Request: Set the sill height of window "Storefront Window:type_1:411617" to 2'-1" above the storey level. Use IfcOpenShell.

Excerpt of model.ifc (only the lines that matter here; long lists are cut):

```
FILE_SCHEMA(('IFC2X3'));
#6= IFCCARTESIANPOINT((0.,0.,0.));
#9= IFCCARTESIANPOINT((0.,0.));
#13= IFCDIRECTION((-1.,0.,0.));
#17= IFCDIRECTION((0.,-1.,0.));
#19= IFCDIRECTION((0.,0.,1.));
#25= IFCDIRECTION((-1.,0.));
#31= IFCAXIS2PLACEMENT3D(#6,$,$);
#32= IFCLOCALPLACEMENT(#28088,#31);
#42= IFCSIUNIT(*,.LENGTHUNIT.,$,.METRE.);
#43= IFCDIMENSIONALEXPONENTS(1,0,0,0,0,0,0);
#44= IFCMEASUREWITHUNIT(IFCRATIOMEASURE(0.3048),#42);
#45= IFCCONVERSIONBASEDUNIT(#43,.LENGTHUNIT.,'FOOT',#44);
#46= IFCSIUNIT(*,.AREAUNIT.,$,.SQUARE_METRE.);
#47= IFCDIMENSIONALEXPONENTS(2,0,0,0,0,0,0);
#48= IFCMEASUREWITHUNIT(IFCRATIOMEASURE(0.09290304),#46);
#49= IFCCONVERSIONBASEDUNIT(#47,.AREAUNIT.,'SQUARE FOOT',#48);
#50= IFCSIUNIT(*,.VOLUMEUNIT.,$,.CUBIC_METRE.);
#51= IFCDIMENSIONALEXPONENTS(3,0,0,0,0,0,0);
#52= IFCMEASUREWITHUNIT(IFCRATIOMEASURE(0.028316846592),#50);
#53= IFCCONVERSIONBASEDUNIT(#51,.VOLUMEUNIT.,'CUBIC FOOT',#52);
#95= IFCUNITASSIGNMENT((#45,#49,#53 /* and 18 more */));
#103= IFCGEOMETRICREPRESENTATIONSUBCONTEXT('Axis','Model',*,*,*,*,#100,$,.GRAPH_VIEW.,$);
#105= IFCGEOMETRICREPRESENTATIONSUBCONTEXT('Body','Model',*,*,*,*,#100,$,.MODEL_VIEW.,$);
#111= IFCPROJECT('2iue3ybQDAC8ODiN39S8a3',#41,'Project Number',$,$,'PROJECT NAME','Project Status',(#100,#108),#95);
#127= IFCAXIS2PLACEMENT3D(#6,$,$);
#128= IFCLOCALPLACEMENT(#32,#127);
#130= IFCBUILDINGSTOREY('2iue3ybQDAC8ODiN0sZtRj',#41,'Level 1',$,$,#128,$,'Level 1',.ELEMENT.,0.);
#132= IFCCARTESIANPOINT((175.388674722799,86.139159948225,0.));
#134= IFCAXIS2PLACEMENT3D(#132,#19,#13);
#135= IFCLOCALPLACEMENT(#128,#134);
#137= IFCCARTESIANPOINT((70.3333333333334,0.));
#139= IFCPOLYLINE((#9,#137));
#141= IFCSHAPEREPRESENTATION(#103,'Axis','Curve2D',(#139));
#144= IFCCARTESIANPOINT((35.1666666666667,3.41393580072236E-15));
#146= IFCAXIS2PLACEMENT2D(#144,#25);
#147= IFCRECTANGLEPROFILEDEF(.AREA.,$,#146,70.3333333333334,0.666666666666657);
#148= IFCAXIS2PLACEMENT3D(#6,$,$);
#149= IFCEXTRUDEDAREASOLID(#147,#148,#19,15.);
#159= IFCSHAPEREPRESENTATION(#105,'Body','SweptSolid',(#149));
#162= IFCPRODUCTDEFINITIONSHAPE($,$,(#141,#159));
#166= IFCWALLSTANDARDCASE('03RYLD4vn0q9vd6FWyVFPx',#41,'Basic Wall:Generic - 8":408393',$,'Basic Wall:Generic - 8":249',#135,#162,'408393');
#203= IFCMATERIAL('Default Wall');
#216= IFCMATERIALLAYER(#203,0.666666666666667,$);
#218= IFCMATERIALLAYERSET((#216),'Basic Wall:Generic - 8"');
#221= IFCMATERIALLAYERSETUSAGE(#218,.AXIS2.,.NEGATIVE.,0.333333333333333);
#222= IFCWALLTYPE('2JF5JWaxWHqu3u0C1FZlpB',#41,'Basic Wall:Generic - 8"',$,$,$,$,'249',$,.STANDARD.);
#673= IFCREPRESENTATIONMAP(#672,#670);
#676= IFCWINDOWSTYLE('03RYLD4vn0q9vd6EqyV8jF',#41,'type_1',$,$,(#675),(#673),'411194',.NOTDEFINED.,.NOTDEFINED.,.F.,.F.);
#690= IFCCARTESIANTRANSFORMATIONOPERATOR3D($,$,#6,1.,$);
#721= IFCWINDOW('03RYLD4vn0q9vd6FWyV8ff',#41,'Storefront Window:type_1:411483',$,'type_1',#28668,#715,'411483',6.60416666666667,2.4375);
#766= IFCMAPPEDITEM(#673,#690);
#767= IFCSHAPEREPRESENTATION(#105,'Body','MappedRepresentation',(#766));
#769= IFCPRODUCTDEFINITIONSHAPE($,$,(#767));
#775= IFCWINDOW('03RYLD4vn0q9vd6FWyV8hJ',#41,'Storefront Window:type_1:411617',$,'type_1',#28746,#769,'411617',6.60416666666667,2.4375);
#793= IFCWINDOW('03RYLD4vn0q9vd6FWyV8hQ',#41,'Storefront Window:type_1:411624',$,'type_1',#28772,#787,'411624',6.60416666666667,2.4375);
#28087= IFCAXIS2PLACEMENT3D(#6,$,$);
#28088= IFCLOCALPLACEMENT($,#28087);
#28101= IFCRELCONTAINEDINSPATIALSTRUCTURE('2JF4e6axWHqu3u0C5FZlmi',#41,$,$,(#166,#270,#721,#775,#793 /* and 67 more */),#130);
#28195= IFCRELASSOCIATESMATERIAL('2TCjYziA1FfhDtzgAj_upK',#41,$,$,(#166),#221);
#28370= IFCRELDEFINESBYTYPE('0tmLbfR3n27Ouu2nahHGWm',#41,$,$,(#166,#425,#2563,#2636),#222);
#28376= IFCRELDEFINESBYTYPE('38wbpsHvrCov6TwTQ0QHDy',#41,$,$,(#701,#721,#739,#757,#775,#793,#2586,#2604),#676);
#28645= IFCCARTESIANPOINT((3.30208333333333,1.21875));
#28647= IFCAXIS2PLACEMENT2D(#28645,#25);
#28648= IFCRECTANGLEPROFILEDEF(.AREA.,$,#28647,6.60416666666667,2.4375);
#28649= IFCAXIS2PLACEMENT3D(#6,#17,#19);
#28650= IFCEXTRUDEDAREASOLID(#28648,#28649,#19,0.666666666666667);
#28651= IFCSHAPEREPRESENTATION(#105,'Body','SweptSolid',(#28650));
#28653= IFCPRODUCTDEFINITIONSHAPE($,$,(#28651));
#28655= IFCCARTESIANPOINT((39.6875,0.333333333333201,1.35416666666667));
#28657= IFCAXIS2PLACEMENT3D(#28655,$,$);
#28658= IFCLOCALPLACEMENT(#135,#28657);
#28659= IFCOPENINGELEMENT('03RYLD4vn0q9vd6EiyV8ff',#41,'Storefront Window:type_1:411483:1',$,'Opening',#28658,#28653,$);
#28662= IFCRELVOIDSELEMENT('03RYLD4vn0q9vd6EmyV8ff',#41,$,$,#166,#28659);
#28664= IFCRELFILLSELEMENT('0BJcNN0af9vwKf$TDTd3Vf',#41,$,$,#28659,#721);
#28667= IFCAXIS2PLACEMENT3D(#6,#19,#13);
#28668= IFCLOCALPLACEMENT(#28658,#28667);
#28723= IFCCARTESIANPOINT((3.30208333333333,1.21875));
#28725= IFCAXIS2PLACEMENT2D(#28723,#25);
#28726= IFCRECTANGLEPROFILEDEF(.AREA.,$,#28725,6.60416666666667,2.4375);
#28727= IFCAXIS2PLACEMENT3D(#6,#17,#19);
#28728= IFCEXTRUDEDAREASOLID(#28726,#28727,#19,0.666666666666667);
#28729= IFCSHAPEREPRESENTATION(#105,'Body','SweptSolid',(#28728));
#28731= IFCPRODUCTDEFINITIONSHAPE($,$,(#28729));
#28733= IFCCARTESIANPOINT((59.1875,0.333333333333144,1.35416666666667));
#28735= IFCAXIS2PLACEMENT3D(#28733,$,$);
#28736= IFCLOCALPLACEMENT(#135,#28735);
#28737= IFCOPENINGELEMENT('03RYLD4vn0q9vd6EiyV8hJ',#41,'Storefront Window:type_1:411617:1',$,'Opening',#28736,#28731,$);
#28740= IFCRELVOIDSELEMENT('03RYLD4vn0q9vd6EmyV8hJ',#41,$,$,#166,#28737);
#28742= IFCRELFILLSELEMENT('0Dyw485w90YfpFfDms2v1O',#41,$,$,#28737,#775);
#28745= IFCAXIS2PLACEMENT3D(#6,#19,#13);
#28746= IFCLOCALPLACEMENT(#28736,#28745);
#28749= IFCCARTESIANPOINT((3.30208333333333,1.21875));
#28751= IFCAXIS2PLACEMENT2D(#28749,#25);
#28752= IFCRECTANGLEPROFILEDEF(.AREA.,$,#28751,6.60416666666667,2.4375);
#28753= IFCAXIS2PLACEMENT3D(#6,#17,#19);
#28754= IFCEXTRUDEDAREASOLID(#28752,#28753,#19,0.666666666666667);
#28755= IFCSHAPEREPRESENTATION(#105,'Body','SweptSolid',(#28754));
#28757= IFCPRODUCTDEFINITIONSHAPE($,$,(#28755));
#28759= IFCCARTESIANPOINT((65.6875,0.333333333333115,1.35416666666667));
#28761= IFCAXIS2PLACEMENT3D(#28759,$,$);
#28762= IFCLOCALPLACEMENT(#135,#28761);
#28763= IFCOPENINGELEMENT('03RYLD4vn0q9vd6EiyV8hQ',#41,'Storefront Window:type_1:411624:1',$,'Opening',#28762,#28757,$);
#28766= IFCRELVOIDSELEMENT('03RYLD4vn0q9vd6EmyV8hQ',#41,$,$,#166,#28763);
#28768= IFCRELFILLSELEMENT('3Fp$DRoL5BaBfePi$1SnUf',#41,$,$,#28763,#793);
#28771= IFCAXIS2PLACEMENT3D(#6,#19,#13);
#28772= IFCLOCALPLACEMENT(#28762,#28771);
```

```python
import numpy as np
import ifcopenshell
import ifcopenshell.api.geometry
import ifcopenshell.geom
import ifcopenshell.util.element
import ifcopenshell.util.placement
import ifcopenshell.util.shape
import ifcopenshell.util.unit

model = ifcopenshell.open("model.ifc")
unit_scale = ifcopenshell.util.unit.calculate_unit_scale(model)

window = model.by_guid("03RYLD4vn0q9vd6FWyV8hJ")
opening = window.FillsVoids[0].RelatingOpeningElement
storey = ifcopenshell.util.element.get_container(window, ifc_class="IfcBuildingStorey")
level = ifcopenshell.util.placement.get_local_placement(storey.ObjectPlacement)[2, 3]

# The opening's origin need not be at the sill, so measure its lowest point.
shape = ifcopenshell.geom.create_shape(ifcopenshell.geom.settings(), opening)
bottom = ifcopenshell.util.shape.get_shape_bottom_elevation(shape, shape.geometry) / unit_scale
dz = level + 25 * 0.0254 / unit_scale - bottom

shift = np.array([0.0, 0.0, dz])
# The window is placed relative to its opening, so it follows when the opening moves.
matrix = ifcopenshell.util.placement.get_local_placement(opening.ObjectPlacement)
matrix[:3, 3] += shift
ifcopenshell.api.geometry.edit_object_placement(
    model, product=opening, matrix=matrix, is_si=False, should_transform_children=True
)

print(f"moved by {dz * unit_scale:+.3f} m")

model.write("model_edited.ifc")
```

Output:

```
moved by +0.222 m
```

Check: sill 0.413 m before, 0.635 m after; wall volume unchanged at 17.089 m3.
